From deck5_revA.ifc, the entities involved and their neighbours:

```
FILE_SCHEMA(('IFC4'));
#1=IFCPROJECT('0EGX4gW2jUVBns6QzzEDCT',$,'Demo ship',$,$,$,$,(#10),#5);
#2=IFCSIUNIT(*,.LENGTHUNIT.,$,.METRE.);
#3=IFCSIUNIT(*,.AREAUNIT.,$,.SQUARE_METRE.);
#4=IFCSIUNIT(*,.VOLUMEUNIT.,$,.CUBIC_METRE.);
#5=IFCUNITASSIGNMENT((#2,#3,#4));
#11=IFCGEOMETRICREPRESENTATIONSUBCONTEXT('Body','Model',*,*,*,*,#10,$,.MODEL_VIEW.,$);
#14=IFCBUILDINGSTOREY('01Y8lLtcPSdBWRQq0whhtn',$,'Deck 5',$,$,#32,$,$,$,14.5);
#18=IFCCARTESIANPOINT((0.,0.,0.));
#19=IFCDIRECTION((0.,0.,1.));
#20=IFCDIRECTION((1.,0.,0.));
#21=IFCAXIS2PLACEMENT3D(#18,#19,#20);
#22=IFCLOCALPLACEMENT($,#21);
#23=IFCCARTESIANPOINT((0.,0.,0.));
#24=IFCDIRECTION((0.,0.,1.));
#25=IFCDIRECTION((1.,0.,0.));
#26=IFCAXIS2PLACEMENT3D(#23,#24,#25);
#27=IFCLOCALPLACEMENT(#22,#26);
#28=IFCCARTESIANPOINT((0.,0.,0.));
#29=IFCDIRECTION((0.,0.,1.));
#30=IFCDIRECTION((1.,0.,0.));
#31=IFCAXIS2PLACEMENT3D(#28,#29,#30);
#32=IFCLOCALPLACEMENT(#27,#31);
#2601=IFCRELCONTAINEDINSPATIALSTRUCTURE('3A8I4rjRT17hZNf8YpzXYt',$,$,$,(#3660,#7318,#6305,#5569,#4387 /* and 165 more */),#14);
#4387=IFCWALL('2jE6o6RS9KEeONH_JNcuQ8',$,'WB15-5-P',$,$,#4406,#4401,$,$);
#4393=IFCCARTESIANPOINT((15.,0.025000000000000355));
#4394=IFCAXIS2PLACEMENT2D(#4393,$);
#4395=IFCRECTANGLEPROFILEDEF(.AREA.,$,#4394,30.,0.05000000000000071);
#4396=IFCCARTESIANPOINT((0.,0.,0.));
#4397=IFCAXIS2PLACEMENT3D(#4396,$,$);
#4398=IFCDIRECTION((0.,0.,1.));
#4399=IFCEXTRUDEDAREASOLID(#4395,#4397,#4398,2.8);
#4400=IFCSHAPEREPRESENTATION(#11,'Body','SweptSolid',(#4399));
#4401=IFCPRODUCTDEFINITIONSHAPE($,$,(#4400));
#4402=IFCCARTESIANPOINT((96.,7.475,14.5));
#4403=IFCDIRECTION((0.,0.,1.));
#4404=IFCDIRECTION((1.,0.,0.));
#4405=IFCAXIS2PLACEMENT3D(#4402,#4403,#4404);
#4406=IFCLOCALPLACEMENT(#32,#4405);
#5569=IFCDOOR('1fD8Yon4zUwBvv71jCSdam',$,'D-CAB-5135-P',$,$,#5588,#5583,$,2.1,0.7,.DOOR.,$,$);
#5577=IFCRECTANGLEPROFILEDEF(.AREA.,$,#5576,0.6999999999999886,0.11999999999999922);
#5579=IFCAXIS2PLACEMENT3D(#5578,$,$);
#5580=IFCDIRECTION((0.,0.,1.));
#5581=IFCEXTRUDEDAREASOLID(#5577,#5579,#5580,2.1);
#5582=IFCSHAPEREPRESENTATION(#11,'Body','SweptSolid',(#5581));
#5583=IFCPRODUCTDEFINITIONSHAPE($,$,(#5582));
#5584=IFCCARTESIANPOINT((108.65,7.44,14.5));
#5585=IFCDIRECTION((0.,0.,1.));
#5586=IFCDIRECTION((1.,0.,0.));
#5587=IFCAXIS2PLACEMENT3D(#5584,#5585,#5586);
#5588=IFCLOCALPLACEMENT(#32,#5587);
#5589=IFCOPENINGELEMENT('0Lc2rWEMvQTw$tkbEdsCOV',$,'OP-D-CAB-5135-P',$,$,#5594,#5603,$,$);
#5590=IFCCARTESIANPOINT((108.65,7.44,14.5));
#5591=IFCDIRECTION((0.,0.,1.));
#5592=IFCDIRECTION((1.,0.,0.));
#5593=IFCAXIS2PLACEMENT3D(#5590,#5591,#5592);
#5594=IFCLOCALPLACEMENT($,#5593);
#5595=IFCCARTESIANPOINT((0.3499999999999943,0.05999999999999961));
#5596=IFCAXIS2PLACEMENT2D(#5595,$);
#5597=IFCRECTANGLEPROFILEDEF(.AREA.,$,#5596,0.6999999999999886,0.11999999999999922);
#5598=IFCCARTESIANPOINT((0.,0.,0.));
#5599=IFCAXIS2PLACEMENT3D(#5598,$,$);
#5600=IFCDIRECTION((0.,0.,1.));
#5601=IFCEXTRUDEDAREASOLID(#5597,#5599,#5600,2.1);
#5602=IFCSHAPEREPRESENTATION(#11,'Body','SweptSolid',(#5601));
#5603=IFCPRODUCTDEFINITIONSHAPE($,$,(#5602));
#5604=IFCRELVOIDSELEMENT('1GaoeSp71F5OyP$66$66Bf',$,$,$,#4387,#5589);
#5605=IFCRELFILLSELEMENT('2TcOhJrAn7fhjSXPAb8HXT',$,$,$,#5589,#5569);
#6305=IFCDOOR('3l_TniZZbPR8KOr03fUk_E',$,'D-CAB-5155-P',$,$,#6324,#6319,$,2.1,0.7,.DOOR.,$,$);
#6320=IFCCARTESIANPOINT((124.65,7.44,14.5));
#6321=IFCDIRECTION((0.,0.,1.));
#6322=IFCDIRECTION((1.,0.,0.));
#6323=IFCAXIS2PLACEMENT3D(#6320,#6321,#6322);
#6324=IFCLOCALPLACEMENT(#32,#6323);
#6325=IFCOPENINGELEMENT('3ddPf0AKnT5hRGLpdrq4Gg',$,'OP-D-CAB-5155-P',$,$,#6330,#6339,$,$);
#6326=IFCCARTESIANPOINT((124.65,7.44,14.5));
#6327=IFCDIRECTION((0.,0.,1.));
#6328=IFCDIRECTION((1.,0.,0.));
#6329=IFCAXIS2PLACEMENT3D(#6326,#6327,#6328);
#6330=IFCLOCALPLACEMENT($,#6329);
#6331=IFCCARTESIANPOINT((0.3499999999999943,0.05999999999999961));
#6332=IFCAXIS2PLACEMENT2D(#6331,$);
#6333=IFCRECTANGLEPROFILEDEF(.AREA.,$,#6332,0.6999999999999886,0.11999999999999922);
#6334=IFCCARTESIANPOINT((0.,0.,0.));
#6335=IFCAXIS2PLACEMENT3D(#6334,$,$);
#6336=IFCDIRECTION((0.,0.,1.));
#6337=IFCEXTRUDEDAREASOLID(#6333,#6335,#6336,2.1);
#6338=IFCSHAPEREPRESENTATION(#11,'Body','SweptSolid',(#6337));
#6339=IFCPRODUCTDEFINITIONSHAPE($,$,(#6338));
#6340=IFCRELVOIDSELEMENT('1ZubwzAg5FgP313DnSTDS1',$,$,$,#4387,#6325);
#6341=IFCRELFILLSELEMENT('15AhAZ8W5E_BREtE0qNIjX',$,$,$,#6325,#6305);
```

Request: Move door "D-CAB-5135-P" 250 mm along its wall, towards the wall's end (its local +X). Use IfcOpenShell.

```python
import ifcopenshell
import ifcopenshell.api.geometry
import ifcopenshell.util.placement
import ifcopenshell.util.unit

model = ifcopenshell.open("deck5_revA.ifc")
unit_scale = ifcopenshell.util.unit.calculate_unit_scale(model)

door = model.by_id(5569)
opening = door.FillsVoids[0].RelatingOpeningElement
wall = opening.VoidsElements[0].RelatingBuildingElement

wall_matrix = ifcopenshell.util.placement.get_local_placement(wall.ObjectPlacement)
shift = wall_matrix[:3, 0] * 0.25 / unit_scale
before = ifcopenshell.util.placement.get_local_placement(door.ObjectPlacement)[:3, 3].copy()

# The door is not placed relative to its opening, so move both.
for product in (opening, door):
    matrix = ifcopenshell.util.placement.get_local_placement(product.ObjectPlacement)
    matrix[:3, 3] += shift
    ifcopenshell.api.geometry.edit_object_placement(model, product=product, matrix=matrix, is_si=False)

after = ifcopenshell.util.placement.get_local_placement(door.ObjectPlacement)[:3, 3]
print("door moved by", (after - before).round(3) + 0.0)

model.write("deck5_revA-out.ifc")
```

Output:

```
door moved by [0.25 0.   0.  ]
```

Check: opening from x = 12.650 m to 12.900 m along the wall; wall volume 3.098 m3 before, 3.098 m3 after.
